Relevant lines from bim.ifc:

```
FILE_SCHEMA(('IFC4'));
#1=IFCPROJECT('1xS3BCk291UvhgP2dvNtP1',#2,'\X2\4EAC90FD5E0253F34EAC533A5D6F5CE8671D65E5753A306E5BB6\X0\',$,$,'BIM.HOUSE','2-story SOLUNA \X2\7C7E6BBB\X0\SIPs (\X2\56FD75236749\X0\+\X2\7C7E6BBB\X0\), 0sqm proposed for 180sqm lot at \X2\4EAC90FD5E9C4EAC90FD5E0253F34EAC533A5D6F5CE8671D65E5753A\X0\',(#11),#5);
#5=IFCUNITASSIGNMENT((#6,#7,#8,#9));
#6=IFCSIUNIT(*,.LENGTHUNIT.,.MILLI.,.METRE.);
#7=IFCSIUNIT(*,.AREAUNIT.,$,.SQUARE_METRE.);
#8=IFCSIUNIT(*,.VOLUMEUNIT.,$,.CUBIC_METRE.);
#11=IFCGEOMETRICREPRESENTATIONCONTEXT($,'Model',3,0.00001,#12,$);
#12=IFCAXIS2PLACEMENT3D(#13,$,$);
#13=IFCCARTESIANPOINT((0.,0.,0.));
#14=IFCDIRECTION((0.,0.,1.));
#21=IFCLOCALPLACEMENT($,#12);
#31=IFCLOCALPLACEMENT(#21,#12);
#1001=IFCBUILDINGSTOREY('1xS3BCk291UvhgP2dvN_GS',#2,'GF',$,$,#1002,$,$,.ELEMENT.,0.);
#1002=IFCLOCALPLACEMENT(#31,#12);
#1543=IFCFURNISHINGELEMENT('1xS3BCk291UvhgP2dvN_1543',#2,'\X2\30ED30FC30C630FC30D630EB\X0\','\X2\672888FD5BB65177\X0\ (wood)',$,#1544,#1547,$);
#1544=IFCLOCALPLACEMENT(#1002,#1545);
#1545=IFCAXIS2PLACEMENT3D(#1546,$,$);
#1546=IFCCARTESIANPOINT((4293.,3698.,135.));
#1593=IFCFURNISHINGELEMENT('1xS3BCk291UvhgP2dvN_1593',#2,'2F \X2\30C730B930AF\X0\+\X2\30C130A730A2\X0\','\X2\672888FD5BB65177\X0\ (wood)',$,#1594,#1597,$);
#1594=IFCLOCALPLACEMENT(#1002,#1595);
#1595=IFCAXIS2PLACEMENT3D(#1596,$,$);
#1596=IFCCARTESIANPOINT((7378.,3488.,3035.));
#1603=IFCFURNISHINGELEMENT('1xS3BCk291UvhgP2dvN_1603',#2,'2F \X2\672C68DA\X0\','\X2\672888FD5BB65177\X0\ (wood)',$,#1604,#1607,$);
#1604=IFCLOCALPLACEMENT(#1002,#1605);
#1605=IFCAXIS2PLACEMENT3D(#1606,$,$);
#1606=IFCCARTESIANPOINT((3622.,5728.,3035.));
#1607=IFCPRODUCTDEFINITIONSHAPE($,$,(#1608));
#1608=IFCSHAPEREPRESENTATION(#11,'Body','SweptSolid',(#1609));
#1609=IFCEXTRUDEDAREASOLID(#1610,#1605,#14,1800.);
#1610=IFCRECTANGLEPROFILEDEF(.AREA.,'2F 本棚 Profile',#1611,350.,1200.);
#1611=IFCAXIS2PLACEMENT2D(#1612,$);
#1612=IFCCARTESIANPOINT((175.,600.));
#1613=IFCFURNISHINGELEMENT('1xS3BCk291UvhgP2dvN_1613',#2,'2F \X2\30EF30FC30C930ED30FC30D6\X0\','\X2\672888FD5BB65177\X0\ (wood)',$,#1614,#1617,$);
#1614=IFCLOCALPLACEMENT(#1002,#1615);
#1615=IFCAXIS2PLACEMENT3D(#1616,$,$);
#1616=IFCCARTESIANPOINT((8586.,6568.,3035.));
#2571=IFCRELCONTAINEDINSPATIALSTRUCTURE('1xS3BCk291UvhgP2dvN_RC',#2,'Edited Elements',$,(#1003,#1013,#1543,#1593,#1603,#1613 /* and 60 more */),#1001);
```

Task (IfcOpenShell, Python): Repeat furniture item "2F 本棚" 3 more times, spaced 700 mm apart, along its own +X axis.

```python
import ifcopenshell
import ifcopenshell.api.geometry
import ifcopenshell.api.root
import ifcopenshell.util.element
import ifcopenshell.util.placement
import ifcopenshell.util.unit

model = ifcopenshell.open("bim.ifc")
unit_scale = ifcopenshell.util.unit.calculate_unit_scale(model)


def reuse_history(source, copy):
    """copy_class also copies each property set's owner history, people and application; keep the originals."""
    for rel in copy.IsDefinedBy:
        if rel.is_a("IfcRelDefinesByProperties") and (history := rel.RelatingPropertyDefinition.OwnerHistory):
            rel.RelatingPropertyDefinition.OwnerHistory = source.OwnerHistory
            ifcopenshell.util.element.remove_deep2(model, history)


source = model.by_id(1603)
base = ifcopenshell.util.placement.get_local_placement(source.ObjectPlacement)
step = base[:3, 0] * 0.7 / unit_scale

for i in range(1, 4):
    copy = ifcopenshell.api.root.copy_class(model, product=source)
    copy.Representation = ifcopenshell.util.element.copy_deep(
        model, source.Representation, exclude=["IfcGeometricRepresentationContext", "IfcRepresentationMap"]
    )
    reuse_history(source, copy)
    matrix = base.copy()
    matrix[:3, 3] += i * step
    print("added at", matrix[:3, 3].round(3) + 0.0)
    ifcopenshell.api.geometry.edit_object_placement(model, product=copy, matrix=matrix, is_si=False)

model.write("bim_edited.ifc")
```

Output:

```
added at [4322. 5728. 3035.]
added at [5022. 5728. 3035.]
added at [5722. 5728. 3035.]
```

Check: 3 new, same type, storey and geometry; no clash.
